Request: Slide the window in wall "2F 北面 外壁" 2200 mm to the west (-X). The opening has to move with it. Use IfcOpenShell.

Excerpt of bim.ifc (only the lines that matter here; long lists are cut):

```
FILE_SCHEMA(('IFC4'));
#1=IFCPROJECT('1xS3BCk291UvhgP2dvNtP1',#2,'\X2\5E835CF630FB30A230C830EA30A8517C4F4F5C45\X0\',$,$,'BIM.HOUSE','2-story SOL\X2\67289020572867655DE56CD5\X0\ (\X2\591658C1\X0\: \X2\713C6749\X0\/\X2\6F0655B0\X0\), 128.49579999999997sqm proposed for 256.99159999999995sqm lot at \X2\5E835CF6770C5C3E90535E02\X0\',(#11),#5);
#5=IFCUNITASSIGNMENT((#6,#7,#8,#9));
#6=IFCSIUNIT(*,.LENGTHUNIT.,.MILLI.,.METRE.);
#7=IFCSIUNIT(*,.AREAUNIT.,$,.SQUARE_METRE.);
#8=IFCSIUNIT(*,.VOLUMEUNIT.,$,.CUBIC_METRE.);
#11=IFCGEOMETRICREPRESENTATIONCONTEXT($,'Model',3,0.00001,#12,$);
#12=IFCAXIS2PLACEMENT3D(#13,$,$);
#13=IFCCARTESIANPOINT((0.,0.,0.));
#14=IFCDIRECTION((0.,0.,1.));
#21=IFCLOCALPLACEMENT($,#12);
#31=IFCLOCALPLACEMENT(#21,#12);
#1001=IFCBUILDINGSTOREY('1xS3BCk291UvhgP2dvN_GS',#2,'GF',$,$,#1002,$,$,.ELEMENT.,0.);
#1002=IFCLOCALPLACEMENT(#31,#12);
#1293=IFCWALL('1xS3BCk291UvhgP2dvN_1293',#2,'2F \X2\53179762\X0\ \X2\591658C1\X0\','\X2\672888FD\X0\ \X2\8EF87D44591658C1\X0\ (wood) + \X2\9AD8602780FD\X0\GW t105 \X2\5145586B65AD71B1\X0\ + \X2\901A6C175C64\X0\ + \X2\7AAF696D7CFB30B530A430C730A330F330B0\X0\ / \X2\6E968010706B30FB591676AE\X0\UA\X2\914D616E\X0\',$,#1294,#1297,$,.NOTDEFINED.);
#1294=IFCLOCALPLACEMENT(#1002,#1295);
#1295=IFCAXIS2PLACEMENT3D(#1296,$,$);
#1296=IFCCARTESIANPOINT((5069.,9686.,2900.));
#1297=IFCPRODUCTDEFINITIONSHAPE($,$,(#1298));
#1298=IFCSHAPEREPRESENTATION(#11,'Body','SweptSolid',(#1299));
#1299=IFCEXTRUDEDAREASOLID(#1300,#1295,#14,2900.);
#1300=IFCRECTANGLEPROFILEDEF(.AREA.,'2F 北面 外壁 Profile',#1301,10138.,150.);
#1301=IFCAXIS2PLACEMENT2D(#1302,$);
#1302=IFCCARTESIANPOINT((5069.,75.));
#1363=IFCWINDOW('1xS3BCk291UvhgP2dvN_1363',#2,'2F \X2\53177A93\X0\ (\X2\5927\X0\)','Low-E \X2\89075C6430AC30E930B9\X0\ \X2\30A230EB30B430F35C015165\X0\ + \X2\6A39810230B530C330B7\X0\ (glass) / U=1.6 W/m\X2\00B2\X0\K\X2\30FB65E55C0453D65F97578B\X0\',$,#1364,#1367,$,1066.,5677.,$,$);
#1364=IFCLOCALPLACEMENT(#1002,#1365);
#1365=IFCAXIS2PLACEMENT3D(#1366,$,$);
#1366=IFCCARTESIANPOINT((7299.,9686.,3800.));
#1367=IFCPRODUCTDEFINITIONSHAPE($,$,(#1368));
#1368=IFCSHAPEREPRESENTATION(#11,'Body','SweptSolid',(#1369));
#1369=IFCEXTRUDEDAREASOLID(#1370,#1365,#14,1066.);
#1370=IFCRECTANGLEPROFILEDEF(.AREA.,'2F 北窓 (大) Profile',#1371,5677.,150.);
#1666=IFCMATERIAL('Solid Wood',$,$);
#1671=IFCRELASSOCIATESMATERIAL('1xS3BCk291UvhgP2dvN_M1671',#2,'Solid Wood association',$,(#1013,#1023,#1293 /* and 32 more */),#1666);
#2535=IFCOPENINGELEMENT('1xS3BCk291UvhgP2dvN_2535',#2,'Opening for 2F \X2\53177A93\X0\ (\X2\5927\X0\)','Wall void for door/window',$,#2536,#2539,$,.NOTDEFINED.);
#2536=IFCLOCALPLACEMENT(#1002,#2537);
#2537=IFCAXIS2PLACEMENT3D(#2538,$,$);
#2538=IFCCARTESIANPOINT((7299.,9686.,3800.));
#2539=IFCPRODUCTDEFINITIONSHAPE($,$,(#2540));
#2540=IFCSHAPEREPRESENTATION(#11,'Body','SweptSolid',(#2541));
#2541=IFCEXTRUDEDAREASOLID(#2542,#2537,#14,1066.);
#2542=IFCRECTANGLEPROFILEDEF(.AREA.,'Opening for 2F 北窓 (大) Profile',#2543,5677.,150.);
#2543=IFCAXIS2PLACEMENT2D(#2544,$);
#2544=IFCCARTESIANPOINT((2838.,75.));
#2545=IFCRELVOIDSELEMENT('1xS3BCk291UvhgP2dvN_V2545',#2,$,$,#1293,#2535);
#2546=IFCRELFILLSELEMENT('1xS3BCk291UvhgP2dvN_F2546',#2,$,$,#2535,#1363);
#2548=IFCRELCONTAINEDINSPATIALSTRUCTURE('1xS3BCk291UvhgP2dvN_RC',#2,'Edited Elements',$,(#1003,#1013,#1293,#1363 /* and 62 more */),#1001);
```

```python
import ifcopenshell
import ifcopenshell.api.geometry
import ifcopenshell.util.placement

model = ifcopenshell.open("bim.ifc")

window = model.by_id(1363)
opening = window.FillsVoids[0].RelatingOpeningElement
wall = opening.VoidsElements[0].RelatingBuildingElement

wall_matrix = ifcopenshell.util.placement.get_local_placement(wall.ObjectPlacement)
shift = wall_matrix[:3, 0] * -2200.0
before = ifcopenshell.util.placement.get_local_placement(window.ObjectPlacement)[:3, 3].copy()

# The window is not placed relative to its opening, so move both.
for product in (opening, window):
    matrix = ifcopenshell.util.placement.get_local_placement(product.ObjectPlacement)
    matrix[:3, 3] += shift
    ifcopenshell.api.geometry.edit_object_placement(model, product=product, matrix=matrix, is_si=False)

after = ifcopenshell.util.placement.get_local_placement(window.ObjectPlacement)[:3, 3]
print("window moved by", (after - before).round(3) + 0.0)

model.write("bim_updated.ifc")
```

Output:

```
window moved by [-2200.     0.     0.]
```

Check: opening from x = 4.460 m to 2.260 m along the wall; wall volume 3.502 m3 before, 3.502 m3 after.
